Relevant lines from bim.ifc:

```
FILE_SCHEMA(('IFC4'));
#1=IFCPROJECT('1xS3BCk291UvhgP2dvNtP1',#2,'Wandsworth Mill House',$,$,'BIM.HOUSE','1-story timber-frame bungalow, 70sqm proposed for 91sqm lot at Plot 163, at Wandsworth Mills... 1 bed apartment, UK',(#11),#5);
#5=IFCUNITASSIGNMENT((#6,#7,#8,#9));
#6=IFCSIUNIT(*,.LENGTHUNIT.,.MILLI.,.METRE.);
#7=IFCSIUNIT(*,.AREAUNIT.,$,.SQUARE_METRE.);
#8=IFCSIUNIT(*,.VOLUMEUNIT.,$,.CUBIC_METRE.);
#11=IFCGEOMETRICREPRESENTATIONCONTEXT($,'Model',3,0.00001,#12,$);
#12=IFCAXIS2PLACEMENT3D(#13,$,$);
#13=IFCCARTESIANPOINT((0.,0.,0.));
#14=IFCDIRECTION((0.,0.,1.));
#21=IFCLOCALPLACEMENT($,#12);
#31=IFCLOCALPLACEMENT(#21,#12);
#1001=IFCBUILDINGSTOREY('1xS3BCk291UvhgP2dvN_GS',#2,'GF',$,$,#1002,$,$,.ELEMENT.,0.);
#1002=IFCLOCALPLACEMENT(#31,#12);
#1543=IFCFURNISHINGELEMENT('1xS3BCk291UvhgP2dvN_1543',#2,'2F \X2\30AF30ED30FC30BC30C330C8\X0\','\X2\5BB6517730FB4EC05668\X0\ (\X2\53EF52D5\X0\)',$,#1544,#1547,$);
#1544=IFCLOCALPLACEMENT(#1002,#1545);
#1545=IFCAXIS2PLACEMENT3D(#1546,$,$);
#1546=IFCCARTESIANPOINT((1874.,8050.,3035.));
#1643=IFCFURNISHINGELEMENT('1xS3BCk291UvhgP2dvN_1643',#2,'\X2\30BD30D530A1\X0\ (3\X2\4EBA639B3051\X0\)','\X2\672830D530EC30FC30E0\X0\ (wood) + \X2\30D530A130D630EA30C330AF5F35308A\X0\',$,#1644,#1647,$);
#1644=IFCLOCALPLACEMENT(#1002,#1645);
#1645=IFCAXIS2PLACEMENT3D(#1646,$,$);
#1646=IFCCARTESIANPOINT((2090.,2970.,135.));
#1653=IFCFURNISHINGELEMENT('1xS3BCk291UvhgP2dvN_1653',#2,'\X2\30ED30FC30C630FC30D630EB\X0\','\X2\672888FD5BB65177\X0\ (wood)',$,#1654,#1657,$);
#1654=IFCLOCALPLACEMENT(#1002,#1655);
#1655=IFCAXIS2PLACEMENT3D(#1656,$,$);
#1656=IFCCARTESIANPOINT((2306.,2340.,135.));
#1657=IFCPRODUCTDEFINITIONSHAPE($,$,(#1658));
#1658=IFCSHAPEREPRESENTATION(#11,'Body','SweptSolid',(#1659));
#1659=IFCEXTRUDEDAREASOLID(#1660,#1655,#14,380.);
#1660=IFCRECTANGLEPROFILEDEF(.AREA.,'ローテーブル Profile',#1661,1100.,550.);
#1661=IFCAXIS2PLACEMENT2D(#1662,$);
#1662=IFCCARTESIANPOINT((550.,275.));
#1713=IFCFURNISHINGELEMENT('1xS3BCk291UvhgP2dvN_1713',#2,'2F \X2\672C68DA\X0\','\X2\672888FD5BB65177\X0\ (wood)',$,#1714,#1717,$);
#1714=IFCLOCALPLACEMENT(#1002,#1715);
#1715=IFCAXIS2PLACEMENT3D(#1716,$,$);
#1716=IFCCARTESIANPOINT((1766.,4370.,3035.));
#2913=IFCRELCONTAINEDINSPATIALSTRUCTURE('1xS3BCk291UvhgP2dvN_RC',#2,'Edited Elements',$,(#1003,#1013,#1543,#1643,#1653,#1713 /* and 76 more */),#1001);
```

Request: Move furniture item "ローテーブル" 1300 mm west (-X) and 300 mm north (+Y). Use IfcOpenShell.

```python
import ifcopenshell
import ifcopenshell.api.geometry
import ifcopenshell.util.placement
import ifcopenshell.util.unit

model = ifcopenshell.open("bim.ifc")
unit_scale = ifcopenshell.util.unit.calculate_unit_scale(model)

item = model.by_guid("1xS3BCk291UvhgP2dvN_1653")
matrix = ifcopenshell.util.placement.get_local_placement(item.ObjectPlacement)
matrix[0, 3] -= 1.3 / unit_scale
matrix[1, 3] += 0.3 / unit_scale
ifcopenshell.api.geometry.edit_object_placement(model, product=item, matrix=matrix, is_si=False)

print(ifcopenshell.util.placement.get_local_placement(item.ObjectPlacement).round(3) + 0.0)

model.write("bim_edited.ifc")
```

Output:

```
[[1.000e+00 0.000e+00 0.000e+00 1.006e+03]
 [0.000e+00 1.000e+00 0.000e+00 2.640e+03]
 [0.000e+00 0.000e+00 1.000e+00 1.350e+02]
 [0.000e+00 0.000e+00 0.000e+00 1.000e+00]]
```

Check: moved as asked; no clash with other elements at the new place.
